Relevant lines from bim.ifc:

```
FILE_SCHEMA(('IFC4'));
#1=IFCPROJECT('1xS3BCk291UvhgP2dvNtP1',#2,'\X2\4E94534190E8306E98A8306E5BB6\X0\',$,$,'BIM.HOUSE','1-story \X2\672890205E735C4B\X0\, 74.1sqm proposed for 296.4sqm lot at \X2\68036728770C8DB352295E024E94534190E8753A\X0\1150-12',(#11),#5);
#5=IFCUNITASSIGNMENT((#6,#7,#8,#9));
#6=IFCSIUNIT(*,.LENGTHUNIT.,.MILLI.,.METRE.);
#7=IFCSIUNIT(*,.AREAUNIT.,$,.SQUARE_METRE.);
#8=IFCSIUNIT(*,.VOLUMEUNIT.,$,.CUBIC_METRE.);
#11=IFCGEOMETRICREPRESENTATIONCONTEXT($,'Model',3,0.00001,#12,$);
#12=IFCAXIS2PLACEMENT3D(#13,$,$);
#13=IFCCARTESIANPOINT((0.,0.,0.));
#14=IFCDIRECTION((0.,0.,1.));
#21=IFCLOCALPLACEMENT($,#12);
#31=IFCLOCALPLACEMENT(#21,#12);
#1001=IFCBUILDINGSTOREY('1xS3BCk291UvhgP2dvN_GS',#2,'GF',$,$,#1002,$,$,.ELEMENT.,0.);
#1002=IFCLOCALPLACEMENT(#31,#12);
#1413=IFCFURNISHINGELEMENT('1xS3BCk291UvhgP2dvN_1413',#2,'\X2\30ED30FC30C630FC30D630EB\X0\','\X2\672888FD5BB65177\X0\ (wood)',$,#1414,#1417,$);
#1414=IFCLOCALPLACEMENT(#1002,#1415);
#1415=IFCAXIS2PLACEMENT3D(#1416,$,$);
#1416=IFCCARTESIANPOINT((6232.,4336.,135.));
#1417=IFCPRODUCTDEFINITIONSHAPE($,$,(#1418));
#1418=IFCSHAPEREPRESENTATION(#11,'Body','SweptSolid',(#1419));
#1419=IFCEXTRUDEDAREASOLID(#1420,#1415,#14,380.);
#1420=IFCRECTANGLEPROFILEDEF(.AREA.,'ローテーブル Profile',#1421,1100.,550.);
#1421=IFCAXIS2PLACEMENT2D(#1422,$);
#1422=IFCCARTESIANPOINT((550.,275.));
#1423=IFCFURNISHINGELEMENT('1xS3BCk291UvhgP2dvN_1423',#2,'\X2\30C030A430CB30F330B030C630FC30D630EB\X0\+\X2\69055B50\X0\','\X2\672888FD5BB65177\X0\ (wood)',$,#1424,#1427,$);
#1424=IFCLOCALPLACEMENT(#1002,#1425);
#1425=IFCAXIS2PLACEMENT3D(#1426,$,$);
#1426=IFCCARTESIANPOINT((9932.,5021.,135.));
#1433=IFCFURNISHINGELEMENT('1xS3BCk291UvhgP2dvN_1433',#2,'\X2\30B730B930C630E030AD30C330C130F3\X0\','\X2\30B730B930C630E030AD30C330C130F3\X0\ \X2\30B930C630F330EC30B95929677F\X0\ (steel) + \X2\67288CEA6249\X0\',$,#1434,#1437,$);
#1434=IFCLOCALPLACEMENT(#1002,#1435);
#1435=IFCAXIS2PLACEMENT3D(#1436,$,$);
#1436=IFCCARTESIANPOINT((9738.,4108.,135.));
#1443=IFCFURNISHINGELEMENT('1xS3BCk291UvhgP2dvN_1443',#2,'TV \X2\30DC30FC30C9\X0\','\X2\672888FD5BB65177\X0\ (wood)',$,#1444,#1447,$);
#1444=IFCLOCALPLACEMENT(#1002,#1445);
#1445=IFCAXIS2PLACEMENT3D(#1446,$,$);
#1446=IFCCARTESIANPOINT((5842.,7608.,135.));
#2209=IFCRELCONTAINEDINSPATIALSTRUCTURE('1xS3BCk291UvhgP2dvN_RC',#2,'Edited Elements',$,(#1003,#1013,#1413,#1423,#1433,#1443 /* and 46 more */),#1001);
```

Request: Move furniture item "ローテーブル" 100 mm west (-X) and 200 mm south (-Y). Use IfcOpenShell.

```python
import ifcopenshell
import ifcopenshell.api.geometry
import ifcopenshell.util.placement

model = ifcopenshell.open("bim.ifc")

item = model.by_guid("1xS3BCk291UvhgP2dvN_1413")
matrix = ifcopenshell.util.placement.get_local_placement(item.ObjectPlacement)
matrix[0, 3] -= 100.0
matrix[1, 3] -= 200.0
ifcopenshell.api.geometry.edit_object_placement(model, product=item, matrix=matrix, is_si=False)

print(ifcopenshell.util.placement.get_local_placement(item.ObjectPlacement).round(3) + 0.0)

model.write("bim_edited.ifc")
```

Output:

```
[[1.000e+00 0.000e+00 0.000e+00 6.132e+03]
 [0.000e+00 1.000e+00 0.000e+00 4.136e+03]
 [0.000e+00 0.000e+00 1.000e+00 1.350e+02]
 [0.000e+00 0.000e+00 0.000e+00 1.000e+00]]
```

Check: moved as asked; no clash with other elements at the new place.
